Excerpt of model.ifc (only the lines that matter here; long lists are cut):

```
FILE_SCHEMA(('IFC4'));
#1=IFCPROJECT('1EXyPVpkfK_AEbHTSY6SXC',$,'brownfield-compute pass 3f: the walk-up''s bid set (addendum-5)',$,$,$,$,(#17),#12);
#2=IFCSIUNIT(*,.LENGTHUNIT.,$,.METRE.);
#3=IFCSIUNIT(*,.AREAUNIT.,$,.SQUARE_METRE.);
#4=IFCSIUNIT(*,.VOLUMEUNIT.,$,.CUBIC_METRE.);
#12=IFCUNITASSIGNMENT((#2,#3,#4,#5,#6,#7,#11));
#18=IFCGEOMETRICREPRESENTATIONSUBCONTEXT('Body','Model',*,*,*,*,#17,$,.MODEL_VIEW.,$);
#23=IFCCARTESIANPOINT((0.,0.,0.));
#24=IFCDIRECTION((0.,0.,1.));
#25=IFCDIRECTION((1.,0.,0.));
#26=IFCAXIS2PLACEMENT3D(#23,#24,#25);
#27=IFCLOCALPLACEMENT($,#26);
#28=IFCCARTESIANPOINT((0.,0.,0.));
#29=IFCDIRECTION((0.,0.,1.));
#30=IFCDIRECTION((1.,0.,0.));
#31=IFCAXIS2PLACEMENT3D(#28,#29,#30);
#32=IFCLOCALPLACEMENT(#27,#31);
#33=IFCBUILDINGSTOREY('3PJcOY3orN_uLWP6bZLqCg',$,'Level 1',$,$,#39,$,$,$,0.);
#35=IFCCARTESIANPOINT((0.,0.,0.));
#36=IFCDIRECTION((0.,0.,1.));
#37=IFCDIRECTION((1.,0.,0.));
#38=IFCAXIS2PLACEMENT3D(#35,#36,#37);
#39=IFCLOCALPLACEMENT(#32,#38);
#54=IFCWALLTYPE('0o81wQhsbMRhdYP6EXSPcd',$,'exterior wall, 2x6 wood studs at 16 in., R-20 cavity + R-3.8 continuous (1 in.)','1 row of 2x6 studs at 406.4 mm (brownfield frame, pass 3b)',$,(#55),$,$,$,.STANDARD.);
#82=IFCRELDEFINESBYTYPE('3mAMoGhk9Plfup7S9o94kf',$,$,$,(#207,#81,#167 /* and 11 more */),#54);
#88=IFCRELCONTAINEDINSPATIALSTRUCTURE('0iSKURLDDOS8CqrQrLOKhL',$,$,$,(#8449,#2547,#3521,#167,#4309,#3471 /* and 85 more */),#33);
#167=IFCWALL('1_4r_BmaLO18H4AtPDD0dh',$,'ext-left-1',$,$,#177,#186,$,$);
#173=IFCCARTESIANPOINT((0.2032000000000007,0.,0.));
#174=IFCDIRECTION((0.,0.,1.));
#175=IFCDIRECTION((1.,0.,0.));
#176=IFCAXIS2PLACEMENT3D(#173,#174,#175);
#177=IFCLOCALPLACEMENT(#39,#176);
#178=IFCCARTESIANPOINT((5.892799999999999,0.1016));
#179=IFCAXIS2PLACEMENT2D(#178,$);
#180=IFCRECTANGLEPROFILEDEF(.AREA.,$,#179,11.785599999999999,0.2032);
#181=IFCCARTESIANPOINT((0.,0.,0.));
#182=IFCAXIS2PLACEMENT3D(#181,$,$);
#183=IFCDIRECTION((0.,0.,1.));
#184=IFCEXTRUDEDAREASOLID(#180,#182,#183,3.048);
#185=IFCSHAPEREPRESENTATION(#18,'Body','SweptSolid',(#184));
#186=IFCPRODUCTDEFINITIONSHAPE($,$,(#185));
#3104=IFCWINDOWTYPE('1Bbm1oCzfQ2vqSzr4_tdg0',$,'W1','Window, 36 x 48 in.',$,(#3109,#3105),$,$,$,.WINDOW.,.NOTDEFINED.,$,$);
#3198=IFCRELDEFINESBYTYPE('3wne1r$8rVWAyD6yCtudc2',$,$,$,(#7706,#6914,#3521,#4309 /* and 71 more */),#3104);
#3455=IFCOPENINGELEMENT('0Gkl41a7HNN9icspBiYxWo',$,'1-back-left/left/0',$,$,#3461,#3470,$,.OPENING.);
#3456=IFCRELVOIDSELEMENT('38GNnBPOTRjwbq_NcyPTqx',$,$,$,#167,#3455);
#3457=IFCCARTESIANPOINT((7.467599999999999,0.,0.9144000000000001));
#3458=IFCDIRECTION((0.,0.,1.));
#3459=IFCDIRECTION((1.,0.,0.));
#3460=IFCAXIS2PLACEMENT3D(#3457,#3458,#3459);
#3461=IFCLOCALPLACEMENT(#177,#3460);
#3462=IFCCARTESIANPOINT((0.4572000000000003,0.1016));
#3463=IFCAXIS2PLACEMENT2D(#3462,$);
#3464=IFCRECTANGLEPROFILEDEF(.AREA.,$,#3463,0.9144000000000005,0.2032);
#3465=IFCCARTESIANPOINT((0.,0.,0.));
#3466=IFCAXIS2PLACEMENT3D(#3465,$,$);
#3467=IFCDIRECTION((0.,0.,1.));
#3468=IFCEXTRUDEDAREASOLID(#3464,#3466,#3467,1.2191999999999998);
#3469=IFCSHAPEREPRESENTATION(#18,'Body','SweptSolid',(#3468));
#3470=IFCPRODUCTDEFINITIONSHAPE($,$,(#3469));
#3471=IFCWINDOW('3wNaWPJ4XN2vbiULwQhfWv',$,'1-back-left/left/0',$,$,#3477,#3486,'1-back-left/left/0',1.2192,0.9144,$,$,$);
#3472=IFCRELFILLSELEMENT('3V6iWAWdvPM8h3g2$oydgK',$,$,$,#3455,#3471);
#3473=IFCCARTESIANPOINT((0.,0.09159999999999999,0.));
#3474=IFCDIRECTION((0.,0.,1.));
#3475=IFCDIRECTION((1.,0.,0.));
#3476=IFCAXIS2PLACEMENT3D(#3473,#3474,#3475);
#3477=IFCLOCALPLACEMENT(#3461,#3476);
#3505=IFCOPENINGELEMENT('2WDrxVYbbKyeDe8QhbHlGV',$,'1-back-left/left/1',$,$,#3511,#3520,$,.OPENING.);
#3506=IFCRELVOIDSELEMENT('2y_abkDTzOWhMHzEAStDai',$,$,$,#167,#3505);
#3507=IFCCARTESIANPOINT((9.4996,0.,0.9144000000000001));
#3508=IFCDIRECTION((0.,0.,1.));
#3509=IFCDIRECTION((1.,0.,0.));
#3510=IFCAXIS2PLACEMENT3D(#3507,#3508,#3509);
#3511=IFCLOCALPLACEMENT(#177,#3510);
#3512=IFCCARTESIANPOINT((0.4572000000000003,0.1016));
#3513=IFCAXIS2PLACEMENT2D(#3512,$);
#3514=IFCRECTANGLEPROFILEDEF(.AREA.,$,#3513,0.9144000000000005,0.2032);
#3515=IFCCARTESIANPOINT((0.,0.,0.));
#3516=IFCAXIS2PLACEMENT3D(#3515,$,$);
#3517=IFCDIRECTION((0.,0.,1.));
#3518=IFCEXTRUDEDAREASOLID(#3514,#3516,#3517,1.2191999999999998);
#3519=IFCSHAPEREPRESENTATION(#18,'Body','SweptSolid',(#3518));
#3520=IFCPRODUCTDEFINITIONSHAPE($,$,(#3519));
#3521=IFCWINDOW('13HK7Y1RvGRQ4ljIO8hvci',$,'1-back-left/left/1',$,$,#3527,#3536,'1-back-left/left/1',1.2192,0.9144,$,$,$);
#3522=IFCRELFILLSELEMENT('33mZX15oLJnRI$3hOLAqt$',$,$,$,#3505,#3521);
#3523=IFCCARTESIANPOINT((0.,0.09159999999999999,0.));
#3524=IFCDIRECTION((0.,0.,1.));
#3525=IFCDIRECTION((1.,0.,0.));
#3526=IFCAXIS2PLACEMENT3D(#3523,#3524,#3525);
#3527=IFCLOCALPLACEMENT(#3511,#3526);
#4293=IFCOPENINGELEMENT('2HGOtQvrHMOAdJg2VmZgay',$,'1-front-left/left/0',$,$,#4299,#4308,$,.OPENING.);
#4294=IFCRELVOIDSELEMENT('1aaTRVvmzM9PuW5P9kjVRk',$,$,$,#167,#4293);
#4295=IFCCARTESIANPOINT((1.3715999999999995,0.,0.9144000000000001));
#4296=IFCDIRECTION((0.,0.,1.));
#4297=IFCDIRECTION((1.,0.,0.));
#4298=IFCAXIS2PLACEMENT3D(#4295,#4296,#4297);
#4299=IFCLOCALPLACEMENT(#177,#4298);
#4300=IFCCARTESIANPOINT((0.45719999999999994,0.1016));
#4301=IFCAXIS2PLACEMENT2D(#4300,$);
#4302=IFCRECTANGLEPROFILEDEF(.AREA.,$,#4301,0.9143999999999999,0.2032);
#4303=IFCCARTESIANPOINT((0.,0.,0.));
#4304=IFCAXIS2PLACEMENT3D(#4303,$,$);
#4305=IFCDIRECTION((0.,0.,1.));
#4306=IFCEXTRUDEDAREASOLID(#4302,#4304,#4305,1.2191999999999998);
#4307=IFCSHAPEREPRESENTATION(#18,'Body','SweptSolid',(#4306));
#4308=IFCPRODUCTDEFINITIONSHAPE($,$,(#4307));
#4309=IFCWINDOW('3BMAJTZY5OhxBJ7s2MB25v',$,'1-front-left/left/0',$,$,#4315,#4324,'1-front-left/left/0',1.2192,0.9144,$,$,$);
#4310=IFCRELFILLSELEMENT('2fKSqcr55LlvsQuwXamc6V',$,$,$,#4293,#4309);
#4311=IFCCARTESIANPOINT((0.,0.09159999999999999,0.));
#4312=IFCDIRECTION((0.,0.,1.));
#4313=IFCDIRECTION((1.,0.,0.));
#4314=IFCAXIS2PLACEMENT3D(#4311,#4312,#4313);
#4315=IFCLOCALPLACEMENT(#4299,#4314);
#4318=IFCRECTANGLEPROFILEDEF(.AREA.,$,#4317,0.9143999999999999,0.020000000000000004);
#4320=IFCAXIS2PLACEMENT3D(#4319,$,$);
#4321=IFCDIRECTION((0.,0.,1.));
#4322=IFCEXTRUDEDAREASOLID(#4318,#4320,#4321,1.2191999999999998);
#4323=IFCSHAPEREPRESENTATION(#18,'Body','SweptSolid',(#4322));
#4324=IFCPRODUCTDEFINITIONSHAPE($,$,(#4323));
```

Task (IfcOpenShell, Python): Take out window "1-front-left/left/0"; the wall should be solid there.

```python
import ifcopenshell
import ifcopenshell.api.feature
import ifcopenshell.api.root
import ifcopenshell.geom
import ifcopenshell.util.shape

model = ifcopenshell.open("model.ifc")
settings = ifcopenshell.geom.settings()


def volume(element):
    """Net volume in cubic metres, openings subtracted."""
    shape = ifcopenshell.geom.create_shape(settings, element)
    return ifcopenshell.util.shape.get_volume(shape.geometry)


window = model.by_guid("3BMAJTZY5OhxBJ7s2MB25v")
opening = window.FillsVoids[0].RelatingOpeningElement
wall = opening.VoidsElements[0].RelatingBuildingElement
before = volume(wall)

ifcopenshell.api.root.remove_product(model, product=window)
ifcopenshell.api.feature.remove_feature(model, feature=opening)

after = volume(wall)

print(f"wall volume {before:.3f} -> {after:.3f} m3")

model.write("model-out.ifc")
```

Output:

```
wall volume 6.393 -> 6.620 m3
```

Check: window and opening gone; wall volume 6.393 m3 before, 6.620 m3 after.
